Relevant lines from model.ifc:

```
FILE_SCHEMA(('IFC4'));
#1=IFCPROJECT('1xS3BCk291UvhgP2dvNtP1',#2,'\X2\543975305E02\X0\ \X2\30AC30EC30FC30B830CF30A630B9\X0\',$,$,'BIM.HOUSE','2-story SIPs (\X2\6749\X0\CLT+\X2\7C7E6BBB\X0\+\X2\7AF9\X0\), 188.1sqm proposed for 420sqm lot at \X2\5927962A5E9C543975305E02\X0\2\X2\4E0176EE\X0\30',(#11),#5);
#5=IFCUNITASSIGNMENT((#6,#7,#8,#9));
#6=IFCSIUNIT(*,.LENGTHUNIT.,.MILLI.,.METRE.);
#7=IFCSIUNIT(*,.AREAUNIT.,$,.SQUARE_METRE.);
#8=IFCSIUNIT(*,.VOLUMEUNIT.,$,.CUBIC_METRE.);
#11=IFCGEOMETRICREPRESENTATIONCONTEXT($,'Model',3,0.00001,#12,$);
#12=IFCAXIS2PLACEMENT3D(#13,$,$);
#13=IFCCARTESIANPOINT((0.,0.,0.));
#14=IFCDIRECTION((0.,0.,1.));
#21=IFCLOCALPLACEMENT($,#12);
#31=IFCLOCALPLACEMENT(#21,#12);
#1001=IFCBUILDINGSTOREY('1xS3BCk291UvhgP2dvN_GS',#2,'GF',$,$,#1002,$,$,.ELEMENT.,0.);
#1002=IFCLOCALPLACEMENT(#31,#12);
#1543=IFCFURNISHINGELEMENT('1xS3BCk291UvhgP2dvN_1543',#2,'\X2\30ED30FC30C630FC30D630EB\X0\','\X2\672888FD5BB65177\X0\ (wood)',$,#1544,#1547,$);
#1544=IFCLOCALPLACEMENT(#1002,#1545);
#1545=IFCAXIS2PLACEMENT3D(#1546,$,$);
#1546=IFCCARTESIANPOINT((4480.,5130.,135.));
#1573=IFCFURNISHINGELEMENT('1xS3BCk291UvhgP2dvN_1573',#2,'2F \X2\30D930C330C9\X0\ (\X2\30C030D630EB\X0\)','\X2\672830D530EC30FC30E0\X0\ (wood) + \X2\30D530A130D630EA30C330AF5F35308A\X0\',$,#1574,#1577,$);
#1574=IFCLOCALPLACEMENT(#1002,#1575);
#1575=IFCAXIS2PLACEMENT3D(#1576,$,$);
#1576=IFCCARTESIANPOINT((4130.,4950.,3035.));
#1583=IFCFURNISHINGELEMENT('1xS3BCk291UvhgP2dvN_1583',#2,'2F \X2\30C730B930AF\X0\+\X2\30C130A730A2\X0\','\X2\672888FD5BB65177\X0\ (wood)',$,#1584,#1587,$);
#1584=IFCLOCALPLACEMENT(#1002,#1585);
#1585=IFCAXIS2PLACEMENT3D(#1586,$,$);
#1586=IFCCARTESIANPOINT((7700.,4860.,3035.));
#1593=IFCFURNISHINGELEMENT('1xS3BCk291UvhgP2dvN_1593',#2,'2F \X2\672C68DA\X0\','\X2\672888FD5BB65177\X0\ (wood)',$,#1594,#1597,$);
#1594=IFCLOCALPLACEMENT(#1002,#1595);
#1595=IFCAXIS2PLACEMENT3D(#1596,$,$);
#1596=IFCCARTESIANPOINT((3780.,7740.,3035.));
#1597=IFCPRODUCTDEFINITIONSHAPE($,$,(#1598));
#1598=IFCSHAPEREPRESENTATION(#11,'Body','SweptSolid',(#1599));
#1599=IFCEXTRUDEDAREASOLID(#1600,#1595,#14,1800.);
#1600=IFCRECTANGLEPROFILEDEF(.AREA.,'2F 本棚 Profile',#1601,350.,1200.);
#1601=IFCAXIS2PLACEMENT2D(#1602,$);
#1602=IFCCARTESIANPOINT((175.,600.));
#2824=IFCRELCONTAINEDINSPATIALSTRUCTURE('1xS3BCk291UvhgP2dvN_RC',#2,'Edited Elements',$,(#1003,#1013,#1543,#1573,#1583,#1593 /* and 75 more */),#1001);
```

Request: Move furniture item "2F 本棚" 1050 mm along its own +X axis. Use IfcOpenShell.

```python
import ifcopenshell
import ifcopenshell.api.geometry
import ifcopenshell.util.placement
import ifcopenshell.util.unit

model = ifcopenshell.open("model.ifc")
unit_scale = ifcopenshell.util.unit.calculate_unit_scale(model)

item = model.by_guid("1xS3BCk291UvhgP2dvN_1593")
matrix = ifcopenshell.util.placement.get_local_placement(item.ObjectPlacement)
matrix[:3, 3] += matrix[:3, 0] * 1.05 / unit_scale
ifcopenshell.api.geometry.edit_object_placement(model, product=item, matrix=matrix, is_si=False)

print(ifcopenshell.util.placement.get_local_placement(item.ObjectPlacement).round(3) + 0.0)

model.write("model_edited.ifc")
```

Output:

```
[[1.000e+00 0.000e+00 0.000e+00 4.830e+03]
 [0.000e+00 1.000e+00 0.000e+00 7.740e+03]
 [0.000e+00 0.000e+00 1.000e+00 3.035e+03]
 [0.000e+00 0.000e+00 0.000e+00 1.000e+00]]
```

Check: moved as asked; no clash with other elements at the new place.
